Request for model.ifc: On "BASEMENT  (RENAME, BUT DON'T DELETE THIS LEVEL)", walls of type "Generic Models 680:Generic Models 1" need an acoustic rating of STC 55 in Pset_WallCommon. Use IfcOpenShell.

First a look at what the model holds.

```python
import ifcopenshell
import ifcopenshell.util.element

model = ifcopenshell.open("model.ifc")
print(model.schema)
storey = next(s for s in model.by_type("IfcBuildingStorey") if s.Name == "BASEMENT  (RENAME, BUT DON'T DELETE THIS LEVEL)")
walls = [e for e in ifcopenshell.util.element.get_decomposition(storey) if e.is_a("IfcWall")]
seen = {}
for e in walls:
    element_type = ifcopenshell.util.element.get_type(e)
    key = (element_type.Name if element_type != e and element_type else None, ifcopenshell.util.element.get_pset(e, "Pset_WallCommon", "AcousticRating"))
    seen[key] = seen.get(key, 0) + 1
for (name, value), count in sorted(seen.items(), key=str):
    print(count, "x", name, "|", value)
```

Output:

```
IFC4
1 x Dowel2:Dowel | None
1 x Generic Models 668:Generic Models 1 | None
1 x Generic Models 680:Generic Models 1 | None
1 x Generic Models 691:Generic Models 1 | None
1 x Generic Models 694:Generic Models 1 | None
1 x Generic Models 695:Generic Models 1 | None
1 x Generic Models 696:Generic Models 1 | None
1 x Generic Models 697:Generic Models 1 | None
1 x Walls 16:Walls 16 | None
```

```python
import ifcopenshell
import ifcopenshell.api.pset
import ifcopenshell.util.element

model = ifcopenshell.open("model.ifc")

storey = next(s for s in model.by_type("IfcBuildingStorey") if s.Name == "BASEMENT  (RENAME, BUT DON'T DELETE THIS LEVEL)")
walls = [e for e in ifcopenshell.util.element.get_decomposition(storey) if e.is_a("IfcWall")]

count = 0
for e in walls:
    element_type = ifcopenshell.util.element.get_type(e)
    if element_type in (None, e) or element_type.Name != "Generic Models 680:Generic Models 1":
        continue
    # add_pset returns the element's existing set when there is one.
    pset = ifcopenshell.api.pset.add_pset(model, product=e, name="Pset_WallCommon")
    ifcopenshell.api.pset.edit_pset(model, pset=pset, properties={"AcousticRating": "STC 55"})
    count += 1

print(count, "walls updated")

model.write("model_v2.ifc")
```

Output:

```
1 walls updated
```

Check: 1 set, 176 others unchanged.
